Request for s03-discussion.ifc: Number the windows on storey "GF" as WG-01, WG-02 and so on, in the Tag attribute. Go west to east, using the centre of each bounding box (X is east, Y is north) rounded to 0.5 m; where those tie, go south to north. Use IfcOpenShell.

First a look at what the model holds.

```python
import ifcopenshell
import ifcopenshell.util.element
import ifcopenshell.util.placement

model = ifcopenshell.open("s03-discussion.ifc")
print(model.schema)
storey = next(s for s in model.by_type("IfcBuildingStorey") if s.Name == "GF")
windows = [e for e in ifcopenshell.util.element.get_decomposition(storey) if e.is_a("IfcWindow")]
for e in sorted(windows, key=lambda e: e.id()):
    origin = ifcopenshell.util.placement.get_local_placement(e.ObjectPlacement)[:3, 3]
    print(e.id(), e.Tag, e.Name, origin.round(2) + 0.0, sep=" | ")
```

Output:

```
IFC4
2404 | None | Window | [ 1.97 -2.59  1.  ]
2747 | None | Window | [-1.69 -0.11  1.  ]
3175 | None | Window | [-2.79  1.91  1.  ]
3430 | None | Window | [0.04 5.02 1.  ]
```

```python
import ifcopenshell
import ifcopenshell.geom
import ifcopenshell.util.element
import ifcopenshell.util.shape

model = ifcopenshell.open("s03-discussion.ifc")
settings = ifcopenshell.geom.settings()
settings.set("use-world-coords", True)


def centre(element):
    shape = ifcopenshell.geom.create_shape(settings, element)
    return ifcopenshell.util.shape.get_bbox_centroid(shape.geometry)


storey = next(s for s in model.by_type("IfcBuildingStorey") if s.Name == "GF")
windows = [e for e in ifcopenshell.util.element.get_decomposition(storey) if e.is_a("IfcWindow")]

# Insertion points can sit at a corner or the storey origin, so sort by the geometry (in metres).
centres = {e: centre(e) for e in windows}
windows.sort(key=lambda e: (round(centres[e][0] / 0.5), centres[e][1]))

for i, e in enumerate(windows, start=1):
    number = f"WG-{i:02d}"
    e.Tag = number
    print(e.id(), number)

model.write("s03-discussion_updated.ifc")
```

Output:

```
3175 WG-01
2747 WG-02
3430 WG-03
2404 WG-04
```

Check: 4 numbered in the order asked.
